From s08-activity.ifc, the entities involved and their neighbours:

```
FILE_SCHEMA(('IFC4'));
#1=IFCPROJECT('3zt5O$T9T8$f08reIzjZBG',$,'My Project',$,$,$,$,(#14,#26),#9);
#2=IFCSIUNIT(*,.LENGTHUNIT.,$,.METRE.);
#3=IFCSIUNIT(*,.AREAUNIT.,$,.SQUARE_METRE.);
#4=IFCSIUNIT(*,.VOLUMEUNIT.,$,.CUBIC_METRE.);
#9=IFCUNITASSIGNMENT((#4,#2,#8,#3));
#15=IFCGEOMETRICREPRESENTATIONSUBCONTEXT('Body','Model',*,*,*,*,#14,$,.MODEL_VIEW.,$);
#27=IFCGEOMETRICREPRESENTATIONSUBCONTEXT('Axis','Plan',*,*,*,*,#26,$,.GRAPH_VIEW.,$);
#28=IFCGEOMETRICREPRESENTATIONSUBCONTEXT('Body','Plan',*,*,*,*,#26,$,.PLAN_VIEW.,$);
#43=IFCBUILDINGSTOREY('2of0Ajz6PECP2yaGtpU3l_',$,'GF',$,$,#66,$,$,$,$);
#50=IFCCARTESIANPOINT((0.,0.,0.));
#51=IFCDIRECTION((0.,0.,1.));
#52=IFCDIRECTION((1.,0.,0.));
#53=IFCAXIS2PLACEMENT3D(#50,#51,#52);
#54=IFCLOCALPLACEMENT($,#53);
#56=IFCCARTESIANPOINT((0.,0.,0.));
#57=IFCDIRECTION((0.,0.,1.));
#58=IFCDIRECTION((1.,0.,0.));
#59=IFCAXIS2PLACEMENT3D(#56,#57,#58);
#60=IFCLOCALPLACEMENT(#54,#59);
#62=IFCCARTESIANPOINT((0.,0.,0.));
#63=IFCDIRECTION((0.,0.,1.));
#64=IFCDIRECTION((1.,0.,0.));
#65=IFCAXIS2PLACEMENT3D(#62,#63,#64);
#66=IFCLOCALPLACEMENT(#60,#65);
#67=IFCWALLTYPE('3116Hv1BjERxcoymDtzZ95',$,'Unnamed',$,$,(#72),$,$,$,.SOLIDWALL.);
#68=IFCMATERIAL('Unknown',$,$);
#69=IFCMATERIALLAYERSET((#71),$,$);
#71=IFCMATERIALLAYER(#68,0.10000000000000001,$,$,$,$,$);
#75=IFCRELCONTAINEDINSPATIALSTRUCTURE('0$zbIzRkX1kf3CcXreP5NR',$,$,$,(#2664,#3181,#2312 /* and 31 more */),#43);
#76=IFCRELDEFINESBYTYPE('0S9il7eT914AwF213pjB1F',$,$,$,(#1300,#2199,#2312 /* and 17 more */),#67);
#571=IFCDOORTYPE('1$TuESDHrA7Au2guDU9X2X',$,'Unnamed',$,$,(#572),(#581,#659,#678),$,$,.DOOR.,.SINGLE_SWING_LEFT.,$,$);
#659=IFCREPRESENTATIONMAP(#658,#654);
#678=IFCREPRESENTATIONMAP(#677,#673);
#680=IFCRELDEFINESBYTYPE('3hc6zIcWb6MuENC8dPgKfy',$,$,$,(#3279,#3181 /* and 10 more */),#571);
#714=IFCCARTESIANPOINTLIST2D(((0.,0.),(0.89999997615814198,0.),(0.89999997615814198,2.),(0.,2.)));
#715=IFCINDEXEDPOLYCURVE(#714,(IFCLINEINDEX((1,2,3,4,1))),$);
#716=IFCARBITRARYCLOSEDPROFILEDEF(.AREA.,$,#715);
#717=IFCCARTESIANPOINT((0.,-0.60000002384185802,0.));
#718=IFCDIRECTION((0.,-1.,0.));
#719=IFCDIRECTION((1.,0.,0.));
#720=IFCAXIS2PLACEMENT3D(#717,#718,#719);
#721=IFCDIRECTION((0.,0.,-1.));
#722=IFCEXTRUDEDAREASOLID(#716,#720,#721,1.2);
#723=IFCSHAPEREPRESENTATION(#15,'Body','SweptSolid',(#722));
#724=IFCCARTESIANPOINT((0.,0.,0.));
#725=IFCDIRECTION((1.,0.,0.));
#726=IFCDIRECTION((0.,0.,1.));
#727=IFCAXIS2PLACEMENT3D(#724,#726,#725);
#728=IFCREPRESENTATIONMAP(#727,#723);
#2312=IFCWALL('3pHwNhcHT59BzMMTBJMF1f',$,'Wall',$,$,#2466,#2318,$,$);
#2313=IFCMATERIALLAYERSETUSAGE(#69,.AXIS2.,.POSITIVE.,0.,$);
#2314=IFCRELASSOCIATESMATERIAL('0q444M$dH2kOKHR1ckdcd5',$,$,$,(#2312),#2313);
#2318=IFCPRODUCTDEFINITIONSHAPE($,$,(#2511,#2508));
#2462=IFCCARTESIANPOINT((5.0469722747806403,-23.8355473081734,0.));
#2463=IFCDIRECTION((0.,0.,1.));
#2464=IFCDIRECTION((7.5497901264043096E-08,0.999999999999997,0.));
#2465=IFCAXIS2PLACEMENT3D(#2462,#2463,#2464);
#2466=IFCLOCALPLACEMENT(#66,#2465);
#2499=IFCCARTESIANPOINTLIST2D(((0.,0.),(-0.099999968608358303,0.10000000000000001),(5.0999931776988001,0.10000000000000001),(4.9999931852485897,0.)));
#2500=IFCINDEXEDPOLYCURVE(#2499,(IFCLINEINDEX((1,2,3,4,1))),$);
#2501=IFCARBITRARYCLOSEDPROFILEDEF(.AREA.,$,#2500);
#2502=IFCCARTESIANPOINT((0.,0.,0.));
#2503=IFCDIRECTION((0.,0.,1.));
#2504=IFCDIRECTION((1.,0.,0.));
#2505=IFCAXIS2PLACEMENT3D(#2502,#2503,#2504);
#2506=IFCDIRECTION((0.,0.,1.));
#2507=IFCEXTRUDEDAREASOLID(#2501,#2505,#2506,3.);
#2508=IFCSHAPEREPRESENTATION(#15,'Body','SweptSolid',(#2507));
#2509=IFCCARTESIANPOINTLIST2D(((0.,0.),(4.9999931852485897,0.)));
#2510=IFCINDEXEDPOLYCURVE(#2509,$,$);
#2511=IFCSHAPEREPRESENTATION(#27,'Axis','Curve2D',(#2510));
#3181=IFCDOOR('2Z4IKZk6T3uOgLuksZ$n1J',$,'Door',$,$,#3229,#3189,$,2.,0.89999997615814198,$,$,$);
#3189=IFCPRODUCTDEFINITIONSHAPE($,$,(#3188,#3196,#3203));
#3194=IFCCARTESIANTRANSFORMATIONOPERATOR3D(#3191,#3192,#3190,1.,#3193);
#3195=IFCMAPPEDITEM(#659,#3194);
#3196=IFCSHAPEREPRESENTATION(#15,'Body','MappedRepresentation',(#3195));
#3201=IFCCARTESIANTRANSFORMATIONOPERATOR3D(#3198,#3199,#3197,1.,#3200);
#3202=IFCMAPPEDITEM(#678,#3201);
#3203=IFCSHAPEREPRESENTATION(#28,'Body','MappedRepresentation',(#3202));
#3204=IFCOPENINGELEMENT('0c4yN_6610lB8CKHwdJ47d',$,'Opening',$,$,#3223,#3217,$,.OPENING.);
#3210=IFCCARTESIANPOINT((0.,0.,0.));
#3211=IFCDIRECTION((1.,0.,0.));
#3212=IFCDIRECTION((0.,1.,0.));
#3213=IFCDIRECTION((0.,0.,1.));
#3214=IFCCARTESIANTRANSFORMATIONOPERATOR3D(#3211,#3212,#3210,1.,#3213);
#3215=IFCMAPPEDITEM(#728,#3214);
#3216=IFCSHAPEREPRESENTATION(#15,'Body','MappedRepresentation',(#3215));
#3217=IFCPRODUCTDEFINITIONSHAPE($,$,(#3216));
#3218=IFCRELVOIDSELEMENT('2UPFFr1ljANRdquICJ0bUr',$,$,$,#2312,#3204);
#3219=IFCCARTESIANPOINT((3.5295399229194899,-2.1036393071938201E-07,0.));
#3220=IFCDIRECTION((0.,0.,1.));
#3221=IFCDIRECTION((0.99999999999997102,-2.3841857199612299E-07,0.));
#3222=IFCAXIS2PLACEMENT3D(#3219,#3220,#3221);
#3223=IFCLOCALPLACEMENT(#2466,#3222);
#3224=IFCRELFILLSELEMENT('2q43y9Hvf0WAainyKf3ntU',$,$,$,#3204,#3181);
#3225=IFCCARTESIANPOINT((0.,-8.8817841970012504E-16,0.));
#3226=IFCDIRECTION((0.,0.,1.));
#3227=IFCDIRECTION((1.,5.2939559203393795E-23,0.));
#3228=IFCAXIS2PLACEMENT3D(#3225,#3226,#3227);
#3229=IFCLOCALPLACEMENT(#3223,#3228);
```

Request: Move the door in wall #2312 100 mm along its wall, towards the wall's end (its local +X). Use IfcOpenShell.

```python
import ifcopenshell
import ifcopenshell.api.geometry
import ifcopenshell.util.placement
import ifcopenshell.util.unit

model = ifcopenshell.open("s08-activity.ifc")
unit_scale = ifcopenshell.util.unit.calculate_unit_scale(model)

door = model.by_id(3181)
opening = door.FillsVoids[0].RelatingOpeningElement
wall = opening.VoidsElements[0].RelatingBuildingElement

wall_matrix = ifcopenshell.util.placement.get_local_placement(wall.ObjectPlacement)
shift = wall_matrix[:3, 0] * 0.1 / unit_scale
before = ifcopenshell.util.placement.get_local_placement(door.ObjectPlacement)[:3, 3].copy()

# The door is placed relative to its opening, so it follows when the opening moves.
matrix = ifcopenshell.util.placement.get_local_placement(opening.ObjectPlacement)
matrix[:3, 3] += shift
ifcopenshell.api.geometry.edit_object_placement(
    model, product=opening, matrix=matrix, is_si=False, should_transform_children=True
)

after = ifcopenshell.util.placement.get_local_placement(door.ObjectPlacement)[:3, 3]
print("door moved by", (after - before).round(3) + 0.0)

model.write("s08-activity-out.ifc")
```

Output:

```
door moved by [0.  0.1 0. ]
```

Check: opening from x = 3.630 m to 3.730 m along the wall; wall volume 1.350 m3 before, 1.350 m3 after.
